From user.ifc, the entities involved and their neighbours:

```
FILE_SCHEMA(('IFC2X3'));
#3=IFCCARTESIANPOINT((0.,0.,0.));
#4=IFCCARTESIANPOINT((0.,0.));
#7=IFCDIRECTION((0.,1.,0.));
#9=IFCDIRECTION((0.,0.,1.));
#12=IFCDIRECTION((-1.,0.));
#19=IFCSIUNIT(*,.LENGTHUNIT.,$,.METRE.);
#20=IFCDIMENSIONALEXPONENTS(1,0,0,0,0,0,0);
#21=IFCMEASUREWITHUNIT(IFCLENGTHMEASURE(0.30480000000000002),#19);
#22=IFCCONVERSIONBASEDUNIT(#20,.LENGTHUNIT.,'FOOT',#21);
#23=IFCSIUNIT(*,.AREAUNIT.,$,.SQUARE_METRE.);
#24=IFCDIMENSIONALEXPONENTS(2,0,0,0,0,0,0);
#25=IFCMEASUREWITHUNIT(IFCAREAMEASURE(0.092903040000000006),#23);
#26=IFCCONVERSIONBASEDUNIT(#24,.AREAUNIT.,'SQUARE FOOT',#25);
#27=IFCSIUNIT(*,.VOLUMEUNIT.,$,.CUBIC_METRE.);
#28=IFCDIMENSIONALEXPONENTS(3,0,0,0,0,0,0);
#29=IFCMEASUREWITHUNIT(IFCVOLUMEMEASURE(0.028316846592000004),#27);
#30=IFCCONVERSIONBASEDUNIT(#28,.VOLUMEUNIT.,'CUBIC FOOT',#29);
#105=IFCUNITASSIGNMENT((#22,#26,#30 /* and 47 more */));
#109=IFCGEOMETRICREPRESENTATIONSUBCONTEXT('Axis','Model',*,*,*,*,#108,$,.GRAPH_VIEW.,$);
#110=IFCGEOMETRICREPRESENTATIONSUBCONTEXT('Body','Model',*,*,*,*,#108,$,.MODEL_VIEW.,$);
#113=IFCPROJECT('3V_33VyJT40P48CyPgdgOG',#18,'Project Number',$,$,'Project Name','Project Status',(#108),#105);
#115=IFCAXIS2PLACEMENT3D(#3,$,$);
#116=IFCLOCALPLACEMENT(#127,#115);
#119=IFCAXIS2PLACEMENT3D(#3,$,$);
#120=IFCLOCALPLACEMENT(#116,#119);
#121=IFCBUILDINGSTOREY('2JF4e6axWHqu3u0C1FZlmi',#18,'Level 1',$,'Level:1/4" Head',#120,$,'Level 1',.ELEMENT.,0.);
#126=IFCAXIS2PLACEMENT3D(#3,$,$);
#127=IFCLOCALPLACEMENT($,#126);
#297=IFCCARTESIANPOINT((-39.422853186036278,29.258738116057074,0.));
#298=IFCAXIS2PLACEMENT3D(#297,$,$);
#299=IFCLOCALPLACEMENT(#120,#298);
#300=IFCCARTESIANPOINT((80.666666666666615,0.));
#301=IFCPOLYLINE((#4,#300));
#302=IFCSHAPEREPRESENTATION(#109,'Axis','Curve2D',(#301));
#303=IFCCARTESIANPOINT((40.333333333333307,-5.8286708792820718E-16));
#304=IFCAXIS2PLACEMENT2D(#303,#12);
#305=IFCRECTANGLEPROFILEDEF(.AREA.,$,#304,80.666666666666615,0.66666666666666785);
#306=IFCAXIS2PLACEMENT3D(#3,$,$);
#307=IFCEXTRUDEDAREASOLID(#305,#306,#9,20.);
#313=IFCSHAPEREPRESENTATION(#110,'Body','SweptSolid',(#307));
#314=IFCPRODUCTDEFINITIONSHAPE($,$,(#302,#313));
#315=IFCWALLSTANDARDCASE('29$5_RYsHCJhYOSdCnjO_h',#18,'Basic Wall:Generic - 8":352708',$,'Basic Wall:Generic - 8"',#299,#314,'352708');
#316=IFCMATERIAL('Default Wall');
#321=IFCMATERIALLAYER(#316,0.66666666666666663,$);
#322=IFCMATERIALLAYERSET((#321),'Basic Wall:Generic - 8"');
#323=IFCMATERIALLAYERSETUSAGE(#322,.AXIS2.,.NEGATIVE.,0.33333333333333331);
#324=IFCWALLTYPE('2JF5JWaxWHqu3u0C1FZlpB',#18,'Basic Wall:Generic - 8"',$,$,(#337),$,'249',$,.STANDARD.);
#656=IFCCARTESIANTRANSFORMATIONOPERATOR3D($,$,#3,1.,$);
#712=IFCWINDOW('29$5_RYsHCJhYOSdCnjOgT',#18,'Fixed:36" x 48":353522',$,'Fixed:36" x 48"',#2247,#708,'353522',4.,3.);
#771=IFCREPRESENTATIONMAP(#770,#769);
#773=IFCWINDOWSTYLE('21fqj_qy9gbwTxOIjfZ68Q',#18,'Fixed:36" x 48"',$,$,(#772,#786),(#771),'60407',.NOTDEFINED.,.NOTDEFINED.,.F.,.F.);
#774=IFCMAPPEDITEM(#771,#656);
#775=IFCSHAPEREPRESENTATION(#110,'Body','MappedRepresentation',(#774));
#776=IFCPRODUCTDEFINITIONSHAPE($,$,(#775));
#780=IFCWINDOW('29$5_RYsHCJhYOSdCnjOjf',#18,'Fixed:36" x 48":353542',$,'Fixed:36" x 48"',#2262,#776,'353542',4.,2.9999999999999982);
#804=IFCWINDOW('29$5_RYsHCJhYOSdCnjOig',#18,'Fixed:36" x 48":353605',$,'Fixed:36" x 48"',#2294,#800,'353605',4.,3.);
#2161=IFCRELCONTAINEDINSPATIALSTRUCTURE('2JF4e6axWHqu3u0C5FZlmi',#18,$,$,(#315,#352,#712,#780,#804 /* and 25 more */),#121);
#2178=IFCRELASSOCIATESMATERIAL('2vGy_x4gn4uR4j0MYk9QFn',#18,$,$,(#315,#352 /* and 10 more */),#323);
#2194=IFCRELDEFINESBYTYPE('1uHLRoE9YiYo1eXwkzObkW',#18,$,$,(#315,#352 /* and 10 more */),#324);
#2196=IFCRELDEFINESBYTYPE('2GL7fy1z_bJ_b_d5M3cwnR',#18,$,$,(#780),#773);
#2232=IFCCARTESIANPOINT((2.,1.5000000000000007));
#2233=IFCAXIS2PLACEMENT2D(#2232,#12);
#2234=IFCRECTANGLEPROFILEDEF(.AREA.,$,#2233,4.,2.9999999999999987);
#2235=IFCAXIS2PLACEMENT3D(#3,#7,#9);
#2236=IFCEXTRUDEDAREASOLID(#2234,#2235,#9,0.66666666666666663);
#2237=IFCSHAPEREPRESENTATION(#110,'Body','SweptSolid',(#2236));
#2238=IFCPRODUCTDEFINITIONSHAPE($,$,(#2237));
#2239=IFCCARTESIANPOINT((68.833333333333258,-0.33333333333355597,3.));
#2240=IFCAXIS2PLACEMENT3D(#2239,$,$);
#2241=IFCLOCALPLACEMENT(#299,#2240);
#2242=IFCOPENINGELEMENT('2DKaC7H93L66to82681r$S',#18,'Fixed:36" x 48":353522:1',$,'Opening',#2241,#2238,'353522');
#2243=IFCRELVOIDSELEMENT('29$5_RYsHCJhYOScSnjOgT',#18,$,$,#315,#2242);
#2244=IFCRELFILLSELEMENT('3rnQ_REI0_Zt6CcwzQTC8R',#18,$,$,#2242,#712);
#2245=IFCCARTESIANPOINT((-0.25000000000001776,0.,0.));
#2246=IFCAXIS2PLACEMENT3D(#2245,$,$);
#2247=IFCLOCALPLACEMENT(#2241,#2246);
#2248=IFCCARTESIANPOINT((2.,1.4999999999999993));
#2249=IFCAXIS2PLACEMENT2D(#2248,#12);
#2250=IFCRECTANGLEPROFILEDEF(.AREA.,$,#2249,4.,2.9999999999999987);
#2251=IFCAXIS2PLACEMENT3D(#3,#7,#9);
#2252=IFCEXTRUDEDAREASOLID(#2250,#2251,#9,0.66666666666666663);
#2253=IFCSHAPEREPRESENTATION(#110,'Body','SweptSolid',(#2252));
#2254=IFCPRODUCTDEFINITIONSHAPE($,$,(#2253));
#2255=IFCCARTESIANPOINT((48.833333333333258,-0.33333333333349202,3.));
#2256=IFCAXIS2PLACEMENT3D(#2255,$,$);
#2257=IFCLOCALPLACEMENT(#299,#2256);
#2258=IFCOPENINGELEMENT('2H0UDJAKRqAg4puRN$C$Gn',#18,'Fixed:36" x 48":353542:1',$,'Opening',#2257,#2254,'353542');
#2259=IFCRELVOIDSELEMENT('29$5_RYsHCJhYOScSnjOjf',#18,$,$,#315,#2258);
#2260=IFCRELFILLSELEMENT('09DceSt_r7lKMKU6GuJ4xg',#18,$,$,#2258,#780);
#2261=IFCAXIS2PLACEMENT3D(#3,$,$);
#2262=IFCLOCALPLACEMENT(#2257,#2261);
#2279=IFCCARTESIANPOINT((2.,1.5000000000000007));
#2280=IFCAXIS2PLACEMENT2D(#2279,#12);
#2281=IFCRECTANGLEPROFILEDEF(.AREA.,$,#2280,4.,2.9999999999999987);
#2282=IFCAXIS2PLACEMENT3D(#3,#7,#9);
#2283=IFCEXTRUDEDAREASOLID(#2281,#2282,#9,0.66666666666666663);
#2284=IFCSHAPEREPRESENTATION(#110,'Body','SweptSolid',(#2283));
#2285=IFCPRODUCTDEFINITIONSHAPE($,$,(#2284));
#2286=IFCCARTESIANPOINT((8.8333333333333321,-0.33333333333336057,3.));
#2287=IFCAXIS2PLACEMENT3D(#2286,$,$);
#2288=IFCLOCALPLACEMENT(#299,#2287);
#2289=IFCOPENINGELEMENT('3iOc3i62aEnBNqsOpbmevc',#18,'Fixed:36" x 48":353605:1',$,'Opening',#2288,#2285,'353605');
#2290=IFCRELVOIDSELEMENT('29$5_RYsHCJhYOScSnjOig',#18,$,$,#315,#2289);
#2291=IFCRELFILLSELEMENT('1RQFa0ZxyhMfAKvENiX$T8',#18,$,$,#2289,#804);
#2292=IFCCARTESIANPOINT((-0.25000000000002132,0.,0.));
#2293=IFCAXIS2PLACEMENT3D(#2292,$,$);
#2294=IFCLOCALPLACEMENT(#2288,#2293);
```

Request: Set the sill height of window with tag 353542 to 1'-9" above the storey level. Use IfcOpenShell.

```python
import numpy as np
import ifcopenshell
import ifcopenshell.api.geometry
import ifcopenshell.geom
import ifcopenshell.util.element
import ifcopenshell.util.placement
import ifcopenshell.util.shape
import ifcopenshell.util.unit

model = ifcopenshell.open("user.ifc")
unit_scale = ifcopenshell.util.unit.calculate_unit_scale(model)

window = model.by_guid("29$5_RYsHCJhYOSdCnjOjf")
opening = window.FillsVoids[0].RelatingOpeningElement
storey = ifcopenshell.util.element.get_container(window, ifc_class="IfcBuildingStorey")
level = ifcopenshell.util.placement.get_local_placement(storey.ObjectPlacement)[2, 3]

# The opening's origin need not be at the sill, so measure its lowest point.
shape = ifcopenshell.geom.create_shape(ifcopenshell.geom.settings(), opening)
bottom = ifcopenshell.util.shape.get_shape_bottom_elevation(shape, shape.geometry) / unit_scale
dz = level + 21 * 0.0254 / unit_scale - bottom

shift = np.array([0.0, 0.0, dz])
# The window is placed relative to its opening, so it follows when the opening moves.
matrix = ifcopenshell.util.placement.get_local_placement(opening.ObjectPlacement)
matrix[:3, 3] += shift
ifcopenshell.api.geometry.edit_object_placement(
    model, product=opening, matrix=matrix, is_si=False, should_transform_children=True
)

print(f"moved by {dz * unit_scale:+.3f} m")

model.write("user_rev.ifc")
```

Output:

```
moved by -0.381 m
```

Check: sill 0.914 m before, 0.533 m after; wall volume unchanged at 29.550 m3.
